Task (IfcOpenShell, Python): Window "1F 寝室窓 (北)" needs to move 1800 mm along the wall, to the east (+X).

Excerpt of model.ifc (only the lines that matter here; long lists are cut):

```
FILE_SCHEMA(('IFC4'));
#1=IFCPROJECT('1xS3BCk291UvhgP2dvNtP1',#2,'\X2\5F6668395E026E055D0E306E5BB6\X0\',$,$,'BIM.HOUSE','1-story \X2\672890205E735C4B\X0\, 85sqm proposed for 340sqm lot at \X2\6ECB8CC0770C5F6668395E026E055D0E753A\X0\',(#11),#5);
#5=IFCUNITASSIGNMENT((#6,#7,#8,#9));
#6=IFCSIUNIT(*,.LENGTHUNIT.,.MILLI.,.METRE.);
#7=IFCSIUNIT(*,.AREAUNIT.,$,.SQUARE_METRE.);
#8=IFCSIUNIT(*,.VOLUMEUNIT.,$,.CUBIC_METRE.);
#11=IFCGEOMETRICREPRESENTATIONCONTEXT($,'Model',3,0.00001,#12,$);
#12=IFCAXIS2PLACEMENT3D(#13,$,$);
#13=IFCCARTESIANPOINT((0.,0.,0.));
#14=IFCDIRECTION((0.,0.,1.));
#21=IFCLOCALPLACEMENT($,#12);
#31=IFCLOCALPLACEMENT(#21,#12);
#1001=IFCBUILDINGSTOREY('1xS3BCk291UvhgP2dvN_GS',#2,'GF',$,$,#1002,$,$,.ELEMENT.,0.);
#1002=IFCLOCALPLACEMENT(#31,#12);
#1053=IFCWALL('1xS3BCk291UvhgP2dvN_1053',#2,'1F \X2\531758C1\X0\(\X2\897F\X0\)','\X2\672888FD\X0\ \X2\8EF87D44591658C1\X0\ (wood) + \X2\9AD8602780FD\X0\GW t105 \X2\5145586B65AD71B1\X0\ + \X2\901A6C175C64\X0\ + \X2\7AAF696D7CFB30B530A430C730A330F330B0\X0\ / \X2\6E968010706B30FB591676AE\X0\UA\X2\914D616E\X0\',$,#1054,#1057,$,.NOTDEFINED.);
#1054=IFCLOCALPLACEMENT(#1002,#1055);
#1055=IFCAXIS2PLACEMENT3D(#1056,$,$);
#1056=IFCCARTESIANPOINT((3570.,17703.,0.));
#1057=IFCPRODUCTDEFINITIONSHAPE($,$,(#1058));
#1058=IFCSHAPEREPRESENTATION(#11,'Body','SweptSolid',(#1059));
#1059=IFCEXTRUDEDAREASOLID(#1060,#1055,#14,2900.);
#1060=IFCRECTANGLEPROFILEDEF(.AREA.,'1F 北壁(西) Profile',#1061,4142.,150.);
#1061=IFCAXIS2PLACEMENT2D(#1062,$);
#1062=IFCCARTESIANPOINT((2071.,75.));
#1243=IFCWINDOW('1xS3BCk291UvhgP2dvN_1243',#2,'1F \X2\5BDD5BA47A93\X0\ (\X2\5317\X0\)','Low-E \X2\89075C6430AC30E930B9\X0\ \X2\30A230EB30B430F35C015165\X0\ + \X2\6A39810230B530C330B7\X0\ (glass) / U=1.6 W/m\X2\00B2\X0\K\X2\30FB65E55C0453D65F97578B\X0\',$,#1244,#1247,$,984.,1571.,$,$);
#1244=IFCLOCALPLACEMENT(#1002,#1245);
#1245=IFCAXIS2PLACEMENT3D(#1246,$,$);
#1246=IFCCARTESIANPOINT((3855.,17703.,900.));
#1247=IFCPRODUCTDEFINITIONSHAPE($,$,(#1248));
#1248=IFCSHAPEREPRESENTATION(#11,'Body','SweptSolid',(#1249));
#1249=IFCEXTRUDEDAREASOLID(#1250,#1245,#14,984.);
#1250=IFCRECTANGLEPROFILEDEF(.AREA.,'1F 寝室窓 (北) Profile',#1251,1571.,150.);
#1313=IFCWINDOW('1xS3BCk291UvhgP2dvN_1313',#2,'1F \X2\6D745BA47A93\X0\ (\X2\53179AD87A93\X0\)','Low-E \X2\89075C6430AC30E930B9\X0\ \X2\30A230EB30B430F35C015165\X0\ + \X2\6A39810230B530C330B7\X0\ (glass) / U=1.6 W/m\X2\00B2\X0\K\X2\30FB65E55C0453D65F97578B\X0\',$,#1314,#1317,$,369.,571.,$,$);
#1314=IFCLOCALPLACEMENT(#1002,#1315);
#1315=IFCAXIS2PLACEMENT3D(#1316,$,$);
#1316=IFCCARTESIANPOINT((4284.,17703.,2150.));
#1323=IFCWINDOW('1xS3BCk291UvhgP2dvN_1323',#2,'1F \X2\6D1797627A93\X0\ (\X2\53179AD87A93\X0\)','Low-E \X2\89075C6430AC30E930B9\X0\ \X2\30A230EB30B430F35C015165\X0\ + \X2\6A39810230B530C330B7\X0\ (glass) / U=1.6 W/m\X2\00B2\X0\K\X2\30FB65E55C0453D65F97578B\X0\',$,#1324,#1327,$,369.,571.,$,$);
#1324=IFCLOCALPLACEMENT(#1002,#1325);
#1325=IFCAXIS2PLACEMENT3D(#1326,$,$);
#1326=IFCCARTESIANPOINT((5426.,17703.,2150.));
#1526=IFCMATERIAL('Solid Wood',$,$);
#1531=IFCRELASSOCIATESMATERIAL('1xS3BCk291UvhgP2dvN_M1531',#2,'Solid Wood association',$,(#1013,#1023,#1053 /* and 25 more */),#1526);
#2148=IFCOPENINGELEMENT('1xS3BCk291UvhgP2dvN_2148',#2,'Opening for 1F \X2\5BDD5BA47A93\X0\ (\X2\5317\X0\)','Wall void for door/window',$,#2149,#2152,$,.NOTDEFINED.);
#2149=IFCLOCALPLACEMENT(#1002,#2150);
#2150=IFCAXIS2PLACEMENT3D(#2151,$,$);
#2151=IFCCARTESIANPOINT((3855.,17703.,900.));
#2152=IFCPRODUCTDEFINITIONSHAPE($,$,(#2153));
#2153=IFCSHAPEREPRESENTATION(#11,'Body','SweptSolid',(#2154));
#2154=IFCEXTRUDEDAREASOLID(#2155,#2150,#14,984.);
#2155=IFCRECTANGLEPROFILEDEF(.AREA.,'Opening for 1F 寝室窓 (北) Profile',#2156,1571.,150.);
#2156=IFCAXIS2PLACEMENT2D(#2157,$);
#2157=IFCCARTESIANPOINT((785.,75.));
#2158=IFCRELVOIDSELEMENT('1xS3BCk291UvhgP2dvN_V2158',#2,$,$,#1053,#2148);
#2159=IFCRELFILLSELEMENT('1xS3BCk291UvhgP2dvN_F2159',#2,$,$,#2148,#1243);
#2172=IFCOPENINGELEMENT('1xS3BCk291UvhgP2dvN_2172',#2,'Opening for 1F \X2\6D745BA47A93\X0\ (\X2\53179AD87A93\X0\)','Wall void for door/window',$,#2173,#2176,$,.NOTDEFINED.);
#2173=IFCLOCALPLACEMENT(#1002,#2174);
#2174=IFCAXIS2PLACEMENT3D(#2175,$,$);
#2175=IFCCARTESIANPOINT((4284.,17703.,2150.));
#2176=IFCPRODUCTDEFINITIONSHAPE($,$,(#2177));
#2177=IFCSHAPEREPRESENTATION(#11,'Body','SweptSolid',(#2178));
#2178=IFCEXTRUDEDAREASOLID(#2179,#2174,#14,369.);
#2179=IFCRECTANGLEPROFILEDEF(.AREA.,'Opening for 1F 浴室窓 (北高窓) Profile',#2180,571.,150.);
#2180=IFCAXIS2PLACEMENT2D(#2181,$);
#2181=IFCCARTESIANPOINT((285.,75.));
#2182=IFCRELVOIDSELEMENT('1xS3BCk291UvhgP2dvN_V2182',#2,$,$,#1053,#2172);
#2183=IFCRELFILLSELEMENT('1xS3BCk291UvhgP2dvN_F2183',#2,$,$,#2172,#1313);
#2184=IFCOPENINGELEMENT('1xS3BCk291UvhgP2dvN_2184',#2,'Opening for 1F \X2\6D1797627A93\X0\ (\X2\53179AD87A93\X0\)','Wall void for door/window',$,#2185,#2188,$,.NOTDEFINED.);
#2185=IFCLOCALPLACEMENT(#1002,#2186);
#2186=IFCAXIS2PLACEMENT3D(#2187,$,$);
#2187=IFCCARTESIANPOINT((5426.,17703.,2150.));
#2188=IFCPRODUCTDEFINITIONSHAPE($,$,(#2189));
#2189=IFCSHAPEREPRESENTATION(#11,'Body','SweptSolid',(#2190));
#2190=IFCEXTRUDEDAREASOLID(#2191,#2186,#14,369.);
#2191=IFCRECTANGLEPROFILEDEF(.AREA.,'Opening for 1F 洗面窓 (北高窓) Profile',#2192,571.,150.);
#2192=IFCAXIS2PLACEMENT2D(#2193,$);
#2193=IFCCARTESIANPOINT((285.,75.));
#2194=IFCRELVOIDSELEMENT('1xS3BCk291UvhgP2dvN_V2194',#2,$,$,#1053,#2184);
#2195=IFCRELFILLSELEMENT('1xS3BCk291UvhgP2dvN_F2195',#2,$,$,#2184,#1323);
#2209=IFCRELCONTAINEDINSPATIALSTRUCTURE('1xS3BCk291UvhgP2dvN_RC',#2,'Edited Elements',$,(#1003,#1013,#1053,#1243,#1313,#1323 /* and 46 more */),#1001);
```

```python
import ifcopenshell
import ifcopenshell.api.geometry
import ifcopenshell.util.placement

model = ifcopenshell.open("model.ifc")

window = model.by_guid("1xS3BCk291UvhgP2dvN_1243")
opening = window.FillsVoids[0].RelatingOpeningElement
wall = opening.VoidsElements[0].RelatingBuildingElement

wall_matrix = ifcopenshell.util.placement.get_local_placement(wall.ObjectPlacement)
shift = wall_matrix[:3, 0] * 1800.0
before = ifcopenshell.util.placement.get_local_placement(window.ObjectPlacement)[:3, 3].copy()

# The window is not placed relative to its opening, so move both.
for product in (opening, window):
    matrix = ifcopenshell.util.placement.get_local_placement(product.ObjectPlacement)
    matrix[:3, 3] += shift
    ifcopenshell.api.geometry.edit_object_placement(model, product=product, matrix=matrix, is_si=False)

after = ifcopenshell.util.placement.get_local_placement(window.ObjectPlacement)[:3, 3]
print("window moved by", (after - before).round(3) + 0.0)

model.write("model_edited.ifc")
```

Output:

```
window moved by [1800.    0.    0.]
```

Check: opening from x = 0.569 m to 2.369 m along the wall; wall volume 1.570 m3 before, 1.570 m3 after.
